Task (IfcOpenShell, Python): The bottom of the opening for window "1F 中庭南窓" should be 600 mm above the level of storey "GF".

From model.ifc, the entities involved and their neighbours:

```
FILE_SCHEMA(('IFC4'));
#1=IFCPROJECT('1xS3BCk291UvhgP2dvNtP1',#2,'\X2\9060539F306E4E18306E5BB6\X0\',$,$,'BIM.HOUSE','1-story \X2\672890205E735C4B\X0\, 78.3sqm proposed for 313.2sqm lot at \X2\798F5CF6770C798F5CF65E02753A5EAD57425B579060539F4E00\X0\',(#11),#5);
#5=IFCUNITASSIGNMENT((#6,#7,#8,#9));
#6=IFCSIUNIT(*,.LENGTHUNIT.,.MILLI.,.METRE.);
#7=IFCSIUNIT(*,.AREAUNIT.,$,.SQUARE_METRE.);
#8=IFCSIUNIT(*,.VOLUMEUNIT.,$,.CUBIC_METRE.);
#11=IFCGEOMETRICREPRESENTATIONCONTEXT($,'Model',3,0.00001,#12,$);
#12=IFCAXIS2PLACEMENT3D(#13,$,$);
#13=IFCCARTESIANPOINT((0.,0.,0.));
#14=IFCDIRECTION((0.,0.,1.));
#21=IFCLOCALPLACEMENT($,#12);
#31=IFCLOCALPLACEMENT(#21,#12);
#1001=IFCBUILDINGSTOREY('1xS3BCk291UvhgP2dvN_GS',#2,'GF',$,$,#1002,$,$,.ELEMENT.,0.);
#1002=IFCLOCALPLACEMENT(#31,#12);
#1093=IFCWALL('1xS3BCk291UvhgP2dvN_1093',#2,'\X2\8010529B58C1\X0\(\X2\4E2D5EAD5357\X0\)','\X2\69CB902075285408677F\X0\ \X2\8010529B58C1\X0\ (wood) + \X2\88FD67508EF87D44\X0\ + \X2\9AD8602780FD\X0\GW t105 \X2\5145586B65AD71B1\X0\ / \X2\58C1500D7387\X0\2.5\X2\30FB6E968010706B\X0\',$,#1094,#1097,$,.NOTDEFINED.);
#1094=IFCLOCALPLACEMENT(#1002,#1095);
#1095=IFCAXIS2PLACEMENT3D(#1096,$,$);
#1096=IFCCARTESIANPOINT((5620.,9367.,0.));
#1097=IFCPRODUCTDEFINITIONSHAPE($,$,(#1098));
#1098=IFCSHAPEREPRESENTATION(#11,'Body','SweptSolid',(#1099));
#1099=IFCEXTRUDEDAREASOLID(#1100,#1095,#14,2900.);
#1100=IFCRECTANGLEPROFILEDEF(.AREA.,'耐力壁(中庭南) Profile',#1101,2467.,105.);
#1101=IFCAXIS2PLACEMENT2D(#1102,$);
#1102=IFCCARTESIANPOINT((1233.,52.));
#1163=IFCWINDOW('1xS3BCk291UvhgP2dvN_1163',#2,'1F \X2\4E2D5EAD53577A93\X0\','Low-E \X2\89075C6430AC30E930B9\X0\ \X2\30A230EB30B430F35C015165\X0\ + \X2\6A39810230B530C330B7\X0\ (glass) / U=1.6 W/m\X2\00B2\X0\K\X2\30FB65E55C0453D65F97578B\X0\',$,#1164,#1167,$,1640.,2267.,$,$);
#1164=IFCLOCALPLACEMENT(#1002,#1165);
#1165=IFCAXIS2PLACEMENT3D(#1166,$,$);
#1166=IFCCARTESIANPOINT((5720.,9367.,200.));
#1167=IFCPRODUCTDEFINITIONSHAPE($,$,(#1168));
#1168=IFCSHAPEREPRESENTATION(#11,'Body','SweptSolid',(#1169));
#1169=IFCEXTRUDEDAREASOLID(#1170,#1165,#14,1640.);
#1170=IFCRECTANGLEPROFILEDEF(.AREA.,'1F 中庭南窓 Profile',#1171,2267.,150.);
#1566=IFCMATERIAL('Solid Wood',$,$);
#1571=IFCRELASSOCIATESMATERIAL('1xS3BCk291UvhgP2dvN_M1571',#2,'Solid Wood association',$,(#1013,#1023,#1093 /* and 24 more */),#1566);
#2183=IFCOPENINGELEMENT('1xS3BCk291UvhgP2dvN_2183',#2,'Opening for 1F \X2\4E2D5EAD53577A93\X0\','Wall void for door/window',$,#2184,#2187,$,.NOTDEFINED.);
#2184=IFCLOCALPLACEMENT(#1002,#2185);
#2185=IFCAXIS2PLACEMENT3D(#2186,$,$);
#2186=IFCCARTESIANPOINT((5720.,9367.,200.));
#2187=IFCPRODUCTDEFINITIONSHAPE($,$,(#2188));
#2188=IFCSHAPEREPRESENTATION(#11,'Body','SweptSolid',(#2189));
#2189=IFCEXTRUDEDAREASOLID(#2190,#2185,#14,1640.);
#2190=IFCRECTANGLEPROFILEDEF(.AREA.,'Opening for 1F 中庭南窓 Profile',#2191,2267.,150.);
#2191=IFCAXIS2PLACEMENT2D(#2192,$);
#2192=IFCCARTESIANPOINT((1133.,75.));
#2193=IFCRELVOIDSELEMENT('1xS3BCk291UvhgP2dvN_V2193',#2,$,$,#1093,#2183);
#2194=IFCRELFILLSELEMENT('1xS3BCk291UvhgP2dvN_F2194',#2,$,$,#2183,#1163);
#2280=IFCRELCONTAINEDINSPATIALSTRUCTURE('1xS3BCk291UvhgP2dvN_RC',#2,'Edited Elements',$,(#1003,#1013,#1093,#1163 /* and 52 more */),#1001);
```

```python
import numpy as np
import ifcopenshell
import ifcopenshell.api.geometry
import ifcopenshell.geom
import ifcopenshell.util.element
import ifcopenshell.util.placement
import ifcopenshell.util.shape
import ifcopenshell.util.unit

model = ifcopenshell.open("model.ifc")
unit_scale = ifcopenshell.util.unit.calculate_unit_scale(model)

window = model.by_guid("1xS3BCk291UvhgP2dvN_1163")
opening = window.FillsVoids[0].RelatingOpeningElement
storey = ifcopenshell.util.element.get_container(window, ifc_class="IfcBuildingStorey")
level = ifcopenshell.util.placement.get_local_placement(storey.ObjectPlacement)[2, 3]

# The opening's origin need not be at the sill, so measure its lowest point.
shape = ifcopenshell.geom.create_shape(ifcopenshell.geom.settings(), opening)
bottom = ifcopenshell.util.shape.get_shape_bottom_elevation(shape, shape.geometry) / unit_scale
dz = level + 600.0 - bottom

shift = np.array([0.0, 0.0, dz])
# The window is not placed relative to its opening, so move both.
for product in (opening, window):
    matrix = ifcopenshell.util.placement.get_local_placement(product.ObjectPlacement)
    matrix[:3, 3] += shift
    ifcopenshell.api.geometry.edit_object_placement(model, product=product, matrix=matrix, is_si=False)

print(f"moved by {dz * unit_scale:+.3f} m")

model.write("model_updated.ifc")
```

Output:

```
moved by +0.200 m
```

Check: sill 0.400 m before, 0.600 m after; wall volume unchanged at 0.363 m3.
